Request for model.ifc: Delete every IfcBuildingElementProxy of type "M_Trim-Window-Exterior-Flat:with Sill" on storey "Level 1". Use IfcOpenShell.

First a look at what the model holds.

```python
import ifcopenshell
import ifcopenshell.util.element

model = ifcopenshell.open("model.ifc")
print(model.schema)
storey = next(s for s in model.by_type("IfcBuildingStorey") if s.Name == "Level 1")
proxies = [e for e in ifcopenshell.util.element.get_decomposition(storey) if e.is_a("IfcBuildingElementProxy")]
seen = {}
for e in proxies:
    element_type = ifcopenshell.util.element.get_type(e)
    name = element_type.Name if element_type not in (None, e) else None
    seen[name] = seen.get(name, 0) + 1
for name, count in sorted(seen.items(), key=str):
    print(count, "x", name)
```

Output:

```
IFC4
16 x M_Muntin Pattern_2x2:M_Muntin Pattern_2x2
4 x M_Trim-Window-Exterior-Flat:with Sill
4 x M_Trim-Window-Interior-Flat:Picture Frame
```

```python
import ifcopenshell
import ifcopenshell.api.root
import ifcopenshell.util.element

model = ifcopenshell.open("model.ifc")

storey = next(s for s in model.by_type("IfcBuildingStorey") if s.Name == "Level 1")
proxies = [e for e in ifcopenshell.util.element.get_decomposition(storey) if e.is_a("IfcBuildingElementProxy")]
targets = [e for e in proxies if (t := ifcopenshell.util.element.get_type(e)) not in (None, e) and t.Name == "M_Trim-Window-Exterior-Flat:with Sill"]

for e in targets:
    ifcopenshell.api.root.remove_product(model, product=e)
print(len(targets), "removed")

model.write("model_v2.ifc")
```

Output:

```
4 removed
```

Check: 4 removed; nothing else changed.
